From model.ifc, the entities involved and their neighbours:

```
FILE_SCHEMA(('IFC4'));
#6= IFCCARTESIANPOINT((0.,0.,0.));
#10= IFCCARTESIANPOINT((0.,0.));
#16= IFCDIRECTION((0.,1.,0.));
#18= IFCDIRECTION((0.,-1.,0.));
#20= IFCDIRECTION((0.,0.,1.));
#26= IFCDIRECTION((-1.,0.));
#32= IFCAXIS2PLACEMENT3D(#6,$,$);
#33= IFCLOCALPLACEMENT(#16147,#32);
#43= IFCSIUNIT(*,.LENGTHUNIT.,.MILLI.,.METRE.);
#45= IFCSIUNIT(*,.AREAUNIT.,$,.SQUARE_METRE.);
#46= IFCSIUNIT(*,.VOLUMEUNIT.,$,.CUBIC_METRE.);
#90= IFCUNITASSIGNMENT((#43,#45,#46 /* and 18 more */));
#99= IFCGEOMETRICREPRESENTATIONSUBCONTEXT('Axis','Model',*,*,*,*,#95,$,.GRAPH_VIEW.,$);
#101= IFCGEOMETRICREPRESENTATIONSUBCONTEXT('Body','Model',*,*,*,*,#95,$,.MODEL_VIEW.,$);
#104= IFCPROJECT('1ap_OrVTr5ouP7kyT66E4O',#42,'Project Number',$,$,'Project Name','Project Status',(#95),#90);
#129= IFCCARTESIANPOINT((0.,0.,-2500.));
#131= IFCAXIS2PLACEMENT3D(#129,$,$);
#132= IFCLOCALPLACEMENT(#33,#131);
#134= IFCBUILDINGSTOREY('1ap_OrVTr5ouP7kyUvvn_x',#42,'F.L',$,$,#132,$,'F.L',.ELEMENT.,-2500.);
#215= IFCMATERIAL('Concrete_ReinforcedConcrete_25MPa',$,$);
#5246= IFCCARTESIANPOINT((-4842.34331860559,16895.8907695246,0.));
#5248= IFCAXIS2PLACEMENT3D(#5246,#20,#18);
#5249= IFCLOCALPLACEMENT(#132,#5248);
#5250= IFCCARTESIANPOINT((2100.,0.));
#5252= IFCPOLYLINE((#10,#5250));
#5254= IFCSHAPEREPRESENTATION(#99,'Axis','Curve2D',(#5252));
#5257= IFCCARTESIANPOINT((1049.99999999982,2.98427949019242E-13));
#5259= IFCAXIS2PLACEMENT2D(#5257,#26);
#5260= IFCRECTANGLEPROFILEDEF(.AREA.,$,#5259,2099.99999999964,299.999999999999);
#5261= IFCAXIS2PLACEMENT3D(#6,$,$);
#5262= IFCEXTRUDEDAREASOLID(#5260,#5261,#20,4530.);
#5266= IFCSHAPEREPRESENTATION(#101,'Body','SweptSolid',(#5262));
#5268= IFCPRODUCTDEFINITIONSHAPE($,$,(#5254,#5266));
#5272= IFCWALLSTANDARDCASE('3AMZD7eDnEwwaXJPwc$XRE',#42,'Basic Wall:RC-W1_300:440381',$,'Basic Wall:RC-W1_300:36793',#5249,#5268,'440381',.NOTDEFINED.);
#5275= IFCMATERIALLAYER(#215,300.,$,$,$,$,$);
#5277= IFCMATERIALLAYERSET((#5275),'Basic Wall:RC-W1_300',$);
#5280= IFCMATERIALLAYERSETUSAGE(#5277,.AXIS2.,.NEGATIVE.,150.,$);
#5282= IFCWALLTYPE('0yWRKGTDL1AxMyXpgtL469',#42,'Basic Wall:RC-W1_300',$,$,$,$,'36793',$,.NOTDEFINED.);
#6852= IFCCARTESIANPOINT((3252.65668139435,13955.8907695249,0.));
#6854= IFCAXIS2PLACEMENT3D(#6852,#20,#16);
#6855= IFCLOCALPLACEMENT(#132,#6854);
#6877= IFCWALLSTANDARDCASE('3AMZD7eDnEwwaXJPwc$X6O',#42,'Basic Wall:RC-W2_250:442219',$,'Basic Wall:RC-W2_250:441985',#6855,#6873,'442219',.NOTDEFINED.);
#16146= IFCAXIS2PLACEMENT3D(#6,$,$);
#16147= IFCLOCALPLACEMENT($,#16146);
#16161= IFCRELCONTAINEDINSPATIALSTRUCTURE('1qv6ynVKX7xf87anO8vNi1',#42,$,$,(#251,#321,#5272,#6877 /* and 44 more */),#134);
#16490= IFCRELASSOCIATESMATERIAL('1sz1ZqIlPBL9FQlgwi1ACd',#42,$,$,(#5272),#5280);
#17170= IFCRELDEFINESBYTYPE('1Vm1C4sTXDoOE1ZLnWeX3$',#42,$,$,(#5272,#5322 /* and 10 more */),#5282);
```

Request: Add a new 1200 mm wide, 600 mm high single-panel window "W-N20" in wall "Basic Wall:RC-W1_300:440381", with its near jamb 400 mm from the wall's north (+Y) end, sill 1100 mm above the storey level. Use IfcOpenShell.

```python
import numpy as np
import ifcopenshell
import ifcopenshell.api.feature
import ifcopenshell.api.geometry
import ifcopenshell.api.root
import ifcopenshell.api.spatial
import ifcopenshell.geom
import ifcopenshell.util.element
import ifcopenshell.util.placement
import ifcopenshell.util.representation
import ifcopenshell.util.shape
import ifcopenshell.util.unit

model = ifcopenshell.open("model.ifc")
unit_scale = ifcopenshell.util.unit.calculate_unit_scale(model)
settings = ifcopenshell.geom.settings()


def volume(element):
    """Net volume in cubic metres, openings subtracted."""
    shape = ifcopenshell.geom.create_shape(settings, element)
    return ifcopenshell.util.shape.get_volume(shape.geometry)


wall = model.by_guid("3AMZD7eDnEwwaXJPwc$XRE")
storey = ifcopenshell.util.element.get_container(wall, ifc_class="IfcBuildingStorey")
context = ifcopenshell.util.representation.get_context(model, "Model", "Body", "MODEL_VIEW")
before = volume(wall)

width, height, from_end, sill = 1.2, 0.6, 0.4, 1.1  # metres

# The wall runs along its own X axis, and the end named is its -X end.
wall_shape = ifcopenshell.geom.create_shape(settings, wall)
x, y, z = ifcopenshell.util.shape.get_vertices(wall_shape.geometry).T
start = x.min() + from_end
face, thickness = float(y.min()), float(y.max() - y.min())
wall_matrix = ifcopenshell.util.placement.get_local_placement(wall.ObjectPlacement)
level = ifcopenshell.util.placement.get_local_placement(storey.ObjectPlacement)[2, 3]


def in_wall(x, y):
    """Placement at x, y metres in the wall's axes, at sill height."""
    matrix = wall_matrix.copy()
    matrix[:, 3] = wall_matrix @ np.array([x / unit_scale, y / unit_scale, 0.0, 1.0])
    matrix[2, 3] = level + sill / unit_scale
    return matrix


# Opening: a box that overshoots both wall faces by 50 mm.
opening = ifcopenshell.api.root.create_entity(model, ifc_class="IfcOpeningElement", predefined_type="OPENING")
box = ifcopenshell.api.geometry.add_wall_representation(
    model, context=context, length=width, height=height, thickness=thickness + 0.1
)
ifcopenshell.api.geometry.assign_representation(model, product=opening, representation=box)
ifcopenshell.api.geometry.edit_object_placement(model, product=opening, matrix=in_wall(start, face - 0.05), is_si=False)
ifcopenshell.api.feature.add_feature(model, feature=opening, element=wall)

window = ifcopenshell.api.root.create_entity(model, ifc_class="IfcWindow", name="W-N20", predefined_type="WINDOW")
window.OverallWidth, window.OverallHeight = width / unit_scale, height / unit_scale
window.PartitioningType = "SINGLE_PANEL"
body = ifcopenshell.api.geometry.add_window_representation(
    model,
    context=context,
    overall_width=window.OverallWidth,
    overall_height=window.OverallHeight,
    partition_type="SINGLE_PANEL",
)
ifcopenshell.api.geometry.assign_representation(model, product=window, representation=body)
ifcopenshell.api.spatial.assign_container(model, products=[window], relating_structure=storey)
ifcopenshell.api.feature.add_filling(model, opening=opening, element=window)

# Centre the window in the wall's thickness.
ifcopenshell.api.geometry.edit_object_placement(model, product=window, matrix=in_wall(start, face), is_si=False)
window_shape = ifcopenshell.geom.create_shape(settings, window)
depth = ifcopenshell.util.shape.get_vertices(window_shape.geometry)[:, 1]
offset = face + thickness / 2 - (depth.min() + depth.max()) / 2
ifcopenshell.api.geometry.edit_object_placement(model, product=window, matrix=in_wall(start, offset), is_si=False)

after = volume(wall)

print(f"wall volume {before:.3f} -> {after:.3f} m3")

model.write("model-out.ifc")
```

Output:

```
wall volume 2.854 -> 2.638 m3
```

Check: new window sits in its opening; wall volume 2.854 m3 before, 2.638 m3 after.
